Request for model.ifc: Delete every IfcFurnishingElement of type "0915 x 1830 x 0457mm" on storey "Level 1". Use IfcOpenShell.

First a look at what the model holds.

```python
import ifcopenshell
import ifcopenshell.util.element

model = ifcopenshell.open("model.ifc")
print(model.schema)
storey = next(s for s in model.by_type("IfcBuildingStorey") if s.Name == "Level 1")
furniture = [e for e in ifcopenshell.util.element.get_decomposition(storey) if e.is_a("IfcFurnishingElement")]
seen = {}
for e in furniture:
    element_type = ifcopenshell.util.element.get_type(e)
    name = element_type.Name if element_type not in (None, e) else None
    seen[name] = seen.get(name, 0) + 1
for name, count in sorted(seen.items(), key=str):
    print(count, "x", name)
```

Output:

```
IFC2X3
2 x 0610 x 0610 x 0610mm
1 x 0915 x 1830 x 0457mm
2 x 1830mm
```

```python
import ifcopenshell
import ifcopenshell.api.root
import ifcopenshell.util.element

model = ifcopenshell.open("model.ifc")

storey = next(s for s in model.by_type("IfcBuildingStorey") if s.Name == "Level 1")
furniture = [e for e in ifcopenshell.util.element.get_decomposition(storey) if e.is_a("IfcFurnishingElement")]
targets = [e for e in furniture if (t := ifcopenshell.util.element.get_type(e)) not in (None, e) and t.Name == "0915 x 1830 x 0457mm"]

for e in targets:
    ifcopenshell.api.root.remove_product(model, product=e)
print(len(targets), "removed")

model.write("model_v2.ifc")
```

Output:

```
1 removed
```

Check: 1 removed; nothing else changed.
